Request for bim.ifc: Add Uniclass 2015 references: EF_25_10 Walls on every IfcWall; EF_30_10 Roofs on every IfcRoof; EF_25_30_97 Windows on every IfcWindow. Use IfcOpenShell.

First a look at what the model holds.

```python
import ifcopenshell

model = ifcopenshell.open("bim.ifc")
print(model.schema)
print("classifications:", [c.Name for c in model.by_type("IfcClassification")])
for ifc_class in ("IfcDoor", "IfcRoof", "IfcStair", "IfcWall", "IfcWindow"):
    print(ifc_class, len(model.by_type(ifc_class)))
```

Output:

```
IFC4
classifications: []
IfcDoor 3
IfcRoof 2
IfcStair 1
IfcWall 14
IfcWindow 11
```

```python
import ifcopenshell
import ifcopenshell.api.classification

model = ifcopenshell.open("bim.ifc")

system = ifcopenshell.api.classification.add_classification(model, classification="Uniclass 2015")

codes = {
    "IfcWall": ("EF_25_10", "Walls"),
    "IfcRoof": ("EF_30_10", "Roofs"),
    "IfcWindow": ("EF_25_30_97", "Windows"),
}
for ifc_class, (code, name) in codes.items():
    products = model.by_type(ifc_class)
    ifcopenshell.api.classification.add_reference(
        model, products=products, classification=system, identification=code, name=name
    )
    print(code, len(products))

model.write("bim_edited.ifc")
```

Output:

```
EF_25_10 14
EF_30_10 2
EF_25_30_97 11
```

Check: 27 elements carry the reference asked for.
